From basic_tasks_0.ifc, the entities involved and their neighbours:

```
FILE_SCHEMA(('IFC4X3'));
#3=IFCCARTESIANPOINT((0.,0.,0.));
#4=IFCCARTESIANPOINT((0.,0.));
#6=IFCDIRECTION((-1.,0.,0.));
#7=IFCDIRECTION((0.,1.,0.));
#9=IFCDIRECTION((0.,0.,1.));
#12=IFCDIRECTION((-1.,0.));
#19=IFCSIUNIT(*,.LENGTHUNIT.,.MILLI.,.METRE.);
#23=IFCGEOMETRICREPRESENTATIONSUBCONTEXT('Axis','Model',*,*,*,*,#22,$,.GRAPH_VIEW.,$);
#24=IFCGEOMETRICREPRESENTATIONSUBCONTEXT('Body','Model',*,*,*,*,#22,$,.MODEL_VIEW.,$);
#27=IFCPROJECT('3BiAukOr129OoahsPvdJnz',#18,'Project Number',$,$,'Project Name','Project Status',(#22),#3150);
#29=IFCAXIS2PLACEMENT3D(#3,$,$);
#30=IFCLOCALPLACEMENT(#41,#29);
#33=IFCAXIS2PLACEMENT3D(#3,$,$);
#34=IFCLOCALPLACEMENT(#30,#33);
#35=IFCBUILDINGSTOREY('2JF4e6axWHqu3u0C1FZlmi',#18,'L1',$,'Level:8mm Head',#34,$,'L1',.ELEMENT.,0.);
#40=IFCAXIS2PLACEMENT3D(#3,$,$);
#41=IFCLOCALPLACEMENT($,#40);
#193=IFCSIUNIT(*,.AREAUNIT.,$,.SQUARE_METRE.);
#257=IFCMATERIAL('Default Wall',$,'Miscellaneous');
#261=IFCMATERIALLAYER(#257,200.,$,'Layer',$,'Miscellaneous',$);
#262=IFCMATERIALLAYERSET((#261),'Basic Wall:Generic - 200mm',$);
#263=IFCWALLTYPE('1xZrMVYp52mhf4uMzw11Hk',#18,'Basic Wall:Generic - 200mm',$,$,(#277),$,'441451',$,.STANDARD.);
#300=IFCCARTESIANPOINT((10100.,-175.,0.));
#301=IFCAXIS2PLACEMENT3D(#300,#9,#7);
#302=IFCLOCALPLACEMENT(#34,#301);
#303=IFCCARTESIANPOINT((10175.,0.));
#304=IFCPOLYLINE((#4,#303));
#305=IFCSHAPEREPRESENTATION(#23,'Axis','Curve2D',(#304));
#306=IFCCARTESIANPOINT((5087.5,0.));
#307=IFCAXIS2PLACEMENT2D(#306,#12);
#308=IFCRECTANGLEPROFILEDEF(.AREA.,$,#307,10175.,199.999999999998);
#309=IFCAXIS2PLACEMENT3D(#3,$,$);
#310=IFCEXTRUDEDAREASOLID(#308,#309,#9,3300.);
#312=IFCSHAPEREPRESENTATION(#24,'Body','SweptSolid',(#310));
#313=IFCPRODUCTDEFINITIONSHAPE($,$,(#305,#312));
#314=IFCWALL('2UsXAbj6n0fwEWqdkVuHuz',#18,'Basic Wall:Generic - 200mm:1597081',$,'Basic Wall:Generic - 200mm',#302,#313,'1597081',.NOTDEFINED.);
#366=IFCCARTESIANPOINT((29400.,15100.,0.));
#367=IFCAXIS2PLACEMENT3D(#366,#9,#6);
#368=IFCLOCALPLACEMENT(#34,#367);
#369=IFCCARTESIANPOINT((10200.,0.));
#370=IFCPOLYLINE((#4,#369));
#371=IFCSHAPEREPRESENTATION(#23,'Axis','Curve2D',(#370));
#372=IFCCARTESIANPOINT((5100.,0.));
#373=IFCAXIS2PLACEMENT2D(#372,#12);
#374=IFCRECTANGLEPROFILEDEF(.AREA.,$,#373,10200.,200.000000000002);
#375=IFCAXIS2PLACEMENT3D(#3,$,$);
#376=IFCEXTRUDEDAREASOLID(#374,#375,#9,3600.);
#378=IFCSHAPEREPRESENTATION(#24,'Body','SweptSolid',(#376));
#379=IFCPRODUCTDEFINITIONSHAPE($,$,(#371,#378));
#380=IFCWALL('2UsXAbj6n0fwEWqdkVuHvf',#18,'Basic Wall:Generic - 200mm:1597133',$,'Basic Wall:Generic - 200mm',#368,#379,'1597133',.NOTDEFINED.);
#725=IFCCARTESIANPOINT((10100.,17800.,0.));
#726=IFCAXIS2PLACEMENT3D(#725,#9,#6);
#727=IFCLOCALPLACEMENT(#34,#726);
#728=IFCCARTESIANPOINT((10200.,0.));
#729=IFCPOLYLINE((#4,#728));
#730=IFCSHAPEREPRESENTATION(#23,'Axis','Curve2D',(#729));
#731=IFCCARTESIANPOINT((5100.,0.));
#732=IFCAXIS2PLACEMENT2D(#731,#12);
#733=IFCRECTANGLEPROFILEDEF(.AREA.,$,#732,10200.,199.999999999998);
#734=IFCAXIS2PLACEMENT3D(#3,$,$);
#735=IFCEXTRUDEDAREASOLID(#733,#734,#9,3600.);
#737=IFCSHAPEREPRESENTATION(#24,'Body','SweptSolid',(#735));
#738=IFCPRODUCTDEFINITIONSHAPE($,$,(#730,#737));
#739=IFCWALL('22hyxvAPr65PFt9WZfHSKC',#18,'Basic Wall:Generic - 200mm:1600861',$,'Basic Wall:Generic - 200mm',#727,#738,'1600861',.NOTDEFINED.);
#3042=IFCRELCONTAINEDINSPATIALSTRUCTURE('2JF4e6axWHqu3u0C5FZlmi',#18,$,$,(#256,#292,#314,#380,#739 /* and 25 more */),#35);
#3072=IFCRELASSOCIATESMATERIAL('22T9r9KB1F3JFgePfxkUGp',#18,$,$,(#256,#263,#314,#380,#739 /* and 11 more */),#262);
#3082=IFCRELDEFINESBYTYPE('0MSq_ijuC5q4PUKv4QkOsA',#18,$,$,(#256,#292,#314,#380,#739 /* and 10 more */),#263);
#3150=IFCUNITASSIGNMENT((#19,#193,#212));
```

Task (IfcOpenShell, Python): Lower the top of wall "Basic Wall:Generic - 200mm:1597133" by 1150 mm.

```python
import ifcopenshell
import ifcopenshell.geom
import ifcopenshell.util.representation
import ifcopenshell.util.shape

model = ifcopenshell.open("basic_tasks_0.ifc")
settings = ifcopenshell.geom.settings()


def volume(element):
    """Net volume in cubic metres, openings subtracted."""
    shape = ifcopenshell.geom.create_shape(settings, element)
    return ifcopenshell.util.shape.get_volume(shape.geometry)


wall = model.by_guid("2UsXAbj6n0fwEWqdkVuHvf")
before = volume(wall)

body = ifcopenshell.util.representation.get_representation(wall, "Model", "Body")
solid = body.Items[0]
old_height = solid.Depth
solid.Depth -= 1150.0
after = volume(wall)

print(f"height {old_height:g} -> {solid.Depth:g}, volume {before:.3f} -> {after:.3f} m3")

model.write("basic_tasks_0_edited.ifc")
```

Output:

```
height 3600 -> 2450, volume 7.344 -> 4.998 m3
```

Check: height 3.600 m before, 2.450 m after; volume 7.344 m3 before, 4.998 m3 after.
